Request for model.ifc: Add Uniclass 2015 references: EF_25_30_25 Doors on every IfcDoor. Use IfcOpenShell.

First a look at what the model holds.

```python
import ifcopenshell

model = ifcopenshell.open("model.ifc")
print(model.schema)
print("classifications:", [c.Name for c in model.by_type("IfcClassification")])
for ifc_class in ("IfcDoor", "IfcRoof", "IfcStair", "IfcWall", "IfcWindow"):
    print(ifc_class, len(model.by_type(ifc_class)))
```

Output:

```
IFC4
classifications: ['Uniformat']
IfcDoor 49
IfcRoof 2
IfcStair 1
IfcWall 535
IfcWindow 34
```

```python
import ifcopenshell
import ifcopenshell.api.classification

model = ifcopenshell.open("model.ifc")

system = ifcopenshell.api.classification.add_classification(model, classification="Uniclass 2015")

codes = {
    "IfcDoor": ("EF_25_30_25", "Doors"),
}
for ifc_class, (code, name) in codes.items():
    products = model.by_type(ifc_class)
    ifcopenshell.api.classification.add_reference(
        model, products=products, classification=system, identification=code, name=name
    )
    print(code, len(products))

model.write("model_updated.ifc")
```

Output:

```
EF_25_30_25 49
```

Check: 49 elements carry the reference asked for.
